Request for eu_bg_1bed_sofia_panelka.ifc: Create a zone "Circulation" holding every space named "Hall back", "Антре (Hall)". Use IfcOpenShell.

First a look at what the model holds.

```python
import ifcopenshell

model = ifcopenshell.open("eu_bg_1bed_sofia_panelka.ifc")
print(model.schema)
seen = {}
for space in model.by_type("IfcSpace"):
    seen[space.LongName] = seen.get(space.LongName, 0) + 1
for name, count in sorted(seen.items(), key=str):
    print(count, "x", name)
print("zones:", [z.Name for z in model.by_type("IfcZone")][:20])
```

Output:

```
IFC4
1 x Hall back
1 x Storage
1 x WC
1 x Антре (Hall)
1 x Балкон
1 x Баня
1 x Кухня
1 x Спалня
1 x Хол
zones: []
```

```python
import ifcopenshell
import ifcopenshell.api.group
import ifcopenshell.api.root

model = ifcopenshell.open("eu_bg_1bed_sofia_panelka.ifc")

names = {"Hall back", "Антре (Hall)"}
spaces = [s for s in model.by_type("IfcSpace") if s.LongName in names]

zone = ifcopenshell.api.root.create_entity(model, ifc_class="IfcZone", name="Circulation")
ifcopenshell.api.group.assign_group(model, products=spaces, group=zone)
print(len(spaces), "spaces in", zone.Name)

model.write("eu_bg_1bed_sofia_panelka_updated.ifc")
```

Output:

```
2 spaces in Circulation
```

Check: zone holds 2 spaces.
